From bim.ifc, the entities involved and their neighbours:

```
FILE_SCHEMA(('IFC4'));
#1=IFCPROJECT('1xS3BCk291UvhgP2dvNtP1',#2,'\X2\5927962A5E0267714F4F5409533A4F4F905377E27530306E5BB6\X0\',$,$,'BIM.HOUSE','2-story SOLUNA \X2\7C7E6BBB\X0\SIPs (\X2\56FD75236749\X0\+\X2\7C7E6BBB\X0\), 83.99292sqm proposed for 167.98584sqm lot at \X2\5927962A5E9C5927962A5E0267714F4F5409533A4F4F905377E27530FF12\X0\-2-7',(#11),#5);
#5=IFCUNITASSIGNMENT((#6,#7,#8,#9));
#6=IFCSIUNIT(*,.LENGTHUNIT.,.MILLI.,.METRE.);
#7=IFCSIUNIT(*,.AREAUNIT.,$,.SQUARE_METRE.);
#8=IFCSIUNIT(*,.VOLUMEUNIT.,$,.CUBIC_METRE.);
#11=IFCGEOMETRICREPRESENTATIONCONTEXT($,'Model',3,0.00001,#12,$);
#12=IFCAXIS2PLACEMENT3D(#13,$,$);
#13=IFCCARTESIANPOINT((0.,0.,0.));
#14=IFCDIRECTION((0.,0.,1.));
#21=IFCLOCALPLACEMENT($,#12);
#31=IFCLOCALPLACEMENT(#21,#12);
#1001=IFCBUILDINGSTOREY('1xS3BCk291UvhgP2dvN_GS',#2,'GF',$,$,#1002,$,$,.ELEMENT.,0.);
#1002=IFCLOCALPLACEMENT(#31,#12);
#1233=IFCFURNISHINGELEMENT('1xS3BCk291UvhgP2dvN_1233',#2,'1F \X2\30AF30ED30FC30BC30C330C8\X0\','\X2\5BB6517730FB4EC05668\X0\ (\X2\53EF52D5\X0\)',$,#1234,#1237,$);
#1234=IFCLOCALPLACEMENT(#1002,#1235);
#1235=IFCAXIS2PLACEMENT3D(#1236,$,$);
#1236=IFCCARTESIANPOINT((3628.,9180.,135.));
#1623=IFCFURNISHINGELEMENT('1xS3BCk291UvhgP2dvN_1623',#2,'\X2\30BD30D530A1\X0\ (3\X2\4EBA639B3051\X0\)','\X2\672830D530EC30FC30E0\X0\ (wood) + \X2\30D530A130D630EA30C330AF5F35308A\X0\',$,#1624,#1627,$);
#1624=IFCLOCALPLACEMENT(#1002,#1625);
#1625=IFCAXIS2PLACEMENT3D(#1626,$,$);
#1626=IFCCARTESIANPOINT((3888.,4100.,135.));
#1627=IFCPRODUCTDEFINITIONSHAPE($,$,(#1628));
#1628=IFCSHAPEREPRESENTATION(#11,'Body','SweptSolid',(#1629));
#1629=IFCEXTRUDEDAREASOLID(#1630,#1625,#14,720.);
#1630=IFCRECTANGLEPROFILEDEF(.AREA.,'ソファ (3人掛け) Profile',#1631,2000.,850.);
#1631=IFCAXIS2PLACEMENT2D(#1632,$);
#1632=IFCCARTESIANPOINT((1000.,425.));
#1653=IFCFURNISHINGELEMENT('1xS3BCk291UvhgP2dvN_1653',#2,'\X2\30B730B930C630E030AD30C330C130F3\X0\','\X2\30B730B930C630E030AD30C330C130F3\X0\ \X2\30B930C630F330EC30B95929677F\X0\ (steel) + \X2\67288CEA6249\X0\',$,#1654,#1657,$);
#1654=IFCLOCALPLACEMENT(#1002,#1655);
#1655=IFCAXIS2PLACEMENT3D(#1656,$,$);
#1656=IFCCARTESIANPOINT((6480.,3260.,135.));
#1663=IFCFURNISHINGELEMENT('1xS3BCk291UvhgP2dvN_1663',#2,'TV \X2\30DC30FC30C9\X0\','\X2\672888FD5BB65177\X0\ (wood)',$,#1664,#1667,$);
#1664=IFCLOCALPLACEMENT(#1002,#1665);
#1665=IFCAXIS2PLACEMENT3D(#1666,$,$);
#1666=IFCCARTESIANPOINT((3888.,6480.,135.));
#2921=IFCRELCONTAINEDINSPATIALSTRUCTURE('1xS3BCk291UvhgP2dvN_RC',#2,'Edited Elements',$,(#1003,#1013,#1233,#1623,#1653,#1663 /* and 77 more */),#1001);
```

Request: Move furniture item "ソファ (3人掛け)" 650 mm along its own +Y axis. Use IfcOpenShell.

```python
import ifcopenshell
import ifcopenshell.api.geometry
import ifcopenshell.util.placement

model = ifcopenshell.open("bim.ifc")

item = model.by_guid("1xS3BCk291UvhgP2dvN_1623")
matrix = ifcopenshell.util.placement.get_local_placement(item.ObjectPlacement)
matrix[:3, 3] += matrix[:3, 1] * 650.0
ifcopenshell.api.geometry.edit_object_placement(model, product=item, matrix=matrix, is_si=False)

print(ifcopenshell.util.placement.get_local_placement(item.ObjectPlacement).round(3) + 0.0)

model.write("bim_edited.ifc")
```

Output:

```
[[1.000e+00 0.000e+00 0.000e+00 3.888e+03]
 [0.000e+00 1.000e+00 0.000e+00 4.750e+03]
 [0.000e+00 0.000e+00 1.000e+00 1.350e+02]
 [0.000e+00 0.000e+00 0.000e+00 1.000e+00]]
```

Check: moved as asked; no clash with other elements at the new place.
